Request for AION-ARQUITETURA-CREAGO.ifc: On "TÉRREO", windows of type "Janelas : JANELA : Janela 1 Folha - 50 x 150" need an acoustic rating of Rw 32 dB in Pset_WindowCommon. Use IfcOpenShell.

First a look at what the model holds.

```python
import ifcopenshell
import ifcopenshell.util.element

model = ifcopenshell.open("AION-ARQUITETURA-CREAGO.ifc")
print(model.schema)
storey = next(s for s in model.by_type("IfcBuildingStorey") if s.Name == "TÉRREO")
windows = [e for e in ifcopenshell.util.element.get_decomposition(storey) if e.is_a("IfcWindow")]
seen = {}
for e in windows:
    element_type = ifcopenshell.util.element.get_type(e)
    key = (element_type.Name if element_type != e and element_type else None, ifcopenshell.util.element.get_pset(e, "Pset_WindowCommon", "AcousticRating"))
    seen[key] = seen.get(key, 0) + 1
for (name, value), count in sorted(seen.items(), key=str):
    print(count, "x", name, "|", value)
```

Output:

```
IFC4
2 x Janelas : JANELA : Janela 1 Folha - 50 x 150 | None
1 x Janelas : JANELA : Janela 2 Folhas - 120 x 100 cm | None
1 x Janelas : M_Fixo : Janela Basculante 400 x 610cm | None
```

```python
import ifcopenshell
import ifcopenshell.api.pset
import ifcopenshell.util.element

model = ifcopenshell.open("AION-ARQUITETURA-CREAGO.ifc")

storey = next(s for s in model.by_type("IfcBuildingStorey") if s.Name == "TÉRREO")
windows = [e for e in ifcopenshell.util.element.get_decomposition(storey) if e.is_a("IfcWindow")]

count = 0
for e in windows:
    element_type = ifcopenshell.util.element.get_type(e)
    if element_type in (None, e) or element_type.Name != "Janelas : JANELA : Janela 1 Folha - 50 x 150":
        continue
    # add_pset returns the element's existing set when there is one.
    pset = ifcopenshell.api.pset.add_pset(model, product=e, name="Pset_WindowCommon")
    ifcopenshell.api.pset.edit_pset(model, pset=pset, properties={"AcousticRating": "Rw 32 dB"})
    count += 1

print(count, "windows updated")

model.write("AION-ARQUITETURA-CREAGO_updated.ifc")
```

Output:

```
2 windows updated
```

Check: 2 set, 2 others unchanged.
